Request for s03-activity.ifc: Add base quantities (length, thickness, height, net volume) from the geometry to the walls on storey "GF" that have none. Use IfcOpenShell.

First a look at what the model holds.

```python
import ifcopenshell
import ifcopenshell.util.element
import ifcopenshell.util.unit

model = ifcopenshell.open("s03-activity.ifc")
print(model.schema)
for unit_type in ("LENGTHUNIT", "AREAUNIT", "VOLUMEUNIT"):
    print(unit_type, ifcopenshell.util.unit.calculate_unit_scale(model, unit_type))
storey = next(s for s in model.by_type("IfcBuildingStorey") if s.Name == "GF")
walls = [e for e in ifcopenshell.util.element.get_decomposition(storey) if e.is_a("IfcWall")]
for e in sorted(walls, key=lambda e: e.id()):
    print(e.id(), e.is_a(), e.Name, list(ifcopenshell.util.element.get_psets(e, qtos_only=True)), sep=" | ")
```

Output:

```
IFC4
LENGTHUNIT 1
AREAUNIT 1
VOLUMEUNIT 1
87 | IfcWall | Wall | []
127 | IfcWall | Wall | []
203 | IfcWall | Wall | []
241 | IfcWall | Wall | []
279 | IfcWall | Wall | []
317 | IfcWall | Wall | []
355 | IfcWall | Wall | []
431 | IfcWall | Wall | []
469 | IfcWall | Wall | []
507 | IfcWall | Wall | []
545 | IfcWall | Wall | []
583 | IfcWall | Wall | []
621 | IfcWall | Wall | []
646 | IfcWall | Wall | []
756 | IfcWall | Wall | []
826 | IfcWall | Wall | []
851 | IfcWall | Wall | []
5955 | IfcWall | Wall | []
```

```python
import ifcopenshell
import ifcopenshell.api.pset
import ifcopenshell.geom
import ifcopenshell.util.element
import ifcopenshell.util.shape
import ifcopenshell.util.unit

model = ifcopenshell.open("s03-activity.ifc")
unit_scale = ifcopenshell.util.unit.calculate_unit_scale(model)
volume_scale = ifcopenshell.util.unit.calculate_unit_scale(model, "VOLUMEUNIT")
settings = ifcopenshell.geom.settings()

storey = next(s for s in model.by_type("IfcBuildingStorey") if s.Name == "GF")
walls = [e for e in ifcopenshell.util.element.get_decomposition(storey) if e.is_a("IfcWall")]

for e in sorted(walls, key=lambda e: e.id()):
    if ifcopenshell.util.element.get_psets(e, qtos_only=True, should_inherit=False):
        continue
    # Geometry comes back in metres, in the element's own axes.
    shape = ifcopenshell.geom.create_shape(settings, e)
    values = {
        "Length": ifcopenshell.util.shape.get_x(shape.geometry) / unit_scale,
        "Width": ifcopenshell.util.shape.get_y(shape.geometry) / unit_scale,
        "Height": ifcopenshell.util.shape.get_z(shape.geometry) / unit_scale,
        "NetVolume": ifcopenshell.util.shape.get_volume(shape.geometry) / volume_scale,
    }
    qto = ifcopenshell.api.pset.add_qto(model, product=e, name="Qto_WallBaseQuantities")
    ifcopenshell.api.pset.edit_qto(model, qto=qto, properties=values)
    print(e.id(), {k: round(v, 3) for k, v in values.items()})

model.write("s03-activity_edited.ifc")
```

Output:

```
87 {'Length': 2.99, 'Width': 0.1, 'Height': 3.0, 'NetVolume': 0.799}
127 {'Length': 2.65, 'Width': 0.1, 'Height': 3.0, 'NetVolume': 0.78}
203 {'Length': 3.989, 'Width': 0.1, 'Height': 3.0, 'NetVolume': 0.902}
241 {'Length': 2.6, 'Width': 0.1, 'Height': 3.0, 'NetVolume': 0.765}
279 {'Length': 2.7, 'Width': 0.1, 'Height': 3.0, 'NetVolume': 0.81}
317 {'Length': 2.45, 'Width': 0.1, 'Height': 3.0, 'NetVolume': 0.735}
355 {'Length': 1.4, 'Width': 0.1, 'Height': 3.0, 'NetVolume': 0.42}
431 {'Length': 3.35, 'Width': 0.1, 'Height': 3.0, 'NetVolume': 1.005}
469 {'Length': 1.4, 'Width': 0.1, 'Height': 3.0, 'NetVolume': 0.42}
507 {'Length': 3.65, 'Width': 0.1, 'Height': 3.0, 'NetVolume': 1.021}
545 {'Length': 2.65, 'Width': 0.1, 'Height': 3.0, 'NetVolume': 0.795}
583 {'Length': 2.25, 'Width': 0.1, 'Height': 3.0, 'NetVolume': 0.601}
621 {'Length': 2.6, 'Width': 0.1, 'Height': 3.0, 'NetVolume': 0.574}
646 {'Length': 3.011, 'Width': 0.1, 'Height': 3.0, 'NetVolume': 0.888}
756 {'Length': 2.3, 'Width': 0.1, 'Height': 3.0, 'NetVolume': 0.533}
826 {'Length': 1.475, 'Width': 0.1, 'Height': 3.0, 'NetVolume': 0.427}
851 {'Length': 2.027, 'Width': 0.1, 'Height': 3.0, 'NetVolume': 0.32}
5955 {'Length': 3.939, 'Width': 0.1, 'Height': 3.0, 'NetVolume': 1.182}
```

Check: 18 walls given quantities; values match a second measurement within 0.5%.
